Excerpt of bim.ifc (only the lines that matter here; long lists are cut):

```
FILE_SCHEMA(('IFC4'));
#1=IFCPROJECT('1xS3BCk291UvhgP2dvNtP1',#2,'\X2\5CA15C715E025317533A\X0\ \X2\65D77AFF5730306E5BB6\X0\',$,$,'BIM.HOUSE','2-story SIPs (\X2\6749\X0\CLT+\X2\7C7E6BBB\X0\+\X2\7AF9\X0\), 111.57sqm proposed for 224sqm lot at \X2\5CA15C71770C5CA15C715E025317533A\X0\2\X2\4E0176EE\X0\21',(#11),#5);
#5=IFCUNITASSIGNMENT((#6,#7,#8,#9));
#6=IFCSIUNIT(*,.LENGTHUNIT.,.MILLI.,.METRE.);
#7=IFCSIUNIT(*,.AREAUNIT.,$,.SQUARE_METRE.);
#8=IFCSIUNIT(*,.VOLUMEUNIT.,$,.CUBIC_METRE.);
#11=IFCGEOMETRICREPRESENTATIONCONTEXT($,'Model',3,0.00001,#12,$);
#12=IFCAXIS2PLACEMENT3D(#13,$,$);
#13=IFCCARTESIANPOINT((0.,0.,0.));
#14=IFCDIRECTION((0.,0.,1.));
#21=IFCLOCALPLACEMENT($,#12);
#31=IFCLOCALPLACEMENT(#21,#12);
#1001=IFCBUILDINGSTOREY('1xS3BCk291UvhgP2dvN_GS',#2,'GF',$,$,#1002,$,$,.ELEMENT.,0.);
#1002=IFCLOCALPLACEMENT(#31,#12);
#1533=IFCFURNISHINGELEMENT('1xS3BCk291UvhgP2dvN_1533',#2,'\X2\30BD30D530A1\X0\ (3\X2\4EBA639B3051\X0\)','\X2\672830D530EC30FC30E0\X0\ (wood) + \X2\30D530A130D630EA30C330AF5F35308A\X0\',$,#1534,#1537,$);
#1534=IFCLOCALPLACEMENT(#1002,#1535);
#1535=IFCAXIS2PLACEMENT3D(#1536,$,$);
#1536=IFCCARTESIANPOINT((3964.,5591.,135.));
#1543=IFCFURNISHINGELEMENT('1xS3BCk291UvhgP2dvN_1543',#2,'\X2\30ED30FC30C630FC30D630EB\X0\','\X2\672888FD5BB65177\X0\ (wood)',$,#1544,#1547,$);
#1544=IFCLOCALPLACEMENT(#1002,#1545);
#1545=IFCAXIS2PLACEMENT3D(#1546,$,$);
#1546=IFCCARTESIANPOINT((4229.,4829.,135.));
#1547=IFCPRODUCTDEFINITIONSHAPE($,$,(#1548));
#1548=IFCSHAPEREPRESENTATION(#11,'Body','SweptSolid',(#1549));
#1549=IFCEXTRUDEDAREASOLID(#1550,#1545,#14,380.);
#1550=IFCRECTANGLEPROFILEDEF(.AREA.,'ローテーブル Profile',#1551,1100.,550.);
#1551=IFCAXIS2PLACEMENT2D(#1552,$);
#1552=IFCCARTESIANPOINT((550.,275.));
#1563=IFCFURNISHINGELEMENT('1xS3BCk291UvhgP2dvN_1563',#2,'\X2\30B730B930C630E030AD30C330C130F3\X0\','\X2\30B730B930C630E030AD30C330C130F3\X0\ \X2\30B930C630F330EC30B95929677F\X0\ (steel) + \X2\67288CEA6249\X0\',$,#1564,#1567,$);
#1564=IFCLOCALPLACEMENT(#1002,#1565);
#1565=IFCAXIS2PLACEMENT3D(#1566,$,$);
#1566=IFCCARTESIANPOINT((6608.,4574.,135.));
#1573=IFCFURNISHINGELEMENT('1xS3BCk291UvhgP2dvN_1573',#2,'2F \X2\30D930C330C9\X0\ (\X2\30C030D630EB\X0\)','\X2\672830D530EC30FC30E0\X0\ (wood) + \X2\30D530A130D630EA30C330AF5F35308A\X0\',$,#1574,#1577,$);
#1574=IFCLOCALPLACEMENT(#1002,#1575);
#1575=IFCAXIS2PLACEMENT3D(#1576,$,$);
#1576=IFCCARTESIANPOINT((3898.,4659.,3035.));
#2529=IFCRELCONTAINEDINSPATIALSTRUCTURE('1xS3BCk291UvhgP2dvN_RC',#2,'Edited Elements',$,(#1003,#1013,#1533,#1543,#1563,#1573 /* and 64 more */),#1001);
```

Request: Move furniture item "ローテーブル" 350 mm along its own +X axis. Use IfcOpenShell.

```python
import ifcopenshell
import ifcopenshell.api.geometry
import ifcopenshell.util.placement
import ifcopenshell.util.unit

model = ifcopenshell.open("bim.ifc")
unit_scale = ifcopenshell.util.unit.calculate_unit_scale(model)

item = model.by_id(1543)
matrix = ifcopenshell.util.placement.get_local_placement(item.ObjectPlacement)
matrix[:3, 3] += matrix[:3, 0] * 0.35 / unit_scale
ifcopenshell.api.geometry.edit_object_placement(model, product=item, matrix=matrix, is_si=False)

print(ifcopenshell.util.placement.get_local_placement(item.ObjectPlacement).round(3) + 0.0)

model.write("bim_v2.ifc")
```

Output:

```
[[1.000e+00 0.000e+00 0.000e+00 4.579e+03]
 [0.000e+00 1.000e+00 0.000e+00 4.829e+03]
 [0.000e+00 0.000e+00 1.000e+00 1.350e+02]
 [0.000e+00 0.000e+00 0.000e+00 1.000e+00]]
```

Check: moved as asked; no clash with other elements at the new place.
